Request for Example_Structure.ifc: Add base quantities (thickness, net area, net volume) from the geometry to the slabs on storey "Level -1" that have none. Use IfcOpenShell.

First a look at what the model holds.

```python
import ifcopenshell
import ifcopenshell.util.element
import ifcopenshell.util.unit

model = ifcopenshell.open("Example_Structure.ifc")
print(model.schema)
for unit_type in ("LENGTHUNIT", "AREAUNIT", "VOLUMEUNIT"):
    print(unit_type, ifcopenshell.util.unit.calculate_unit_scale(model, unit_type))
storey = next(s for s in model.by_type("IfcBuildingStorey") if s.Name == "Level -1")
slabs = [e for e in ifcopenshell.util.element.get_decomposition(storey) if e.is_a("IfcSlab")]
for e in sorted(slabs, key=lambda e: e.id()):
    print(e.id(), e.is_a(), e.Name, list(ifcopenshell.util.element.get_psets(e, qtos_only=True)), sep=" | ")
```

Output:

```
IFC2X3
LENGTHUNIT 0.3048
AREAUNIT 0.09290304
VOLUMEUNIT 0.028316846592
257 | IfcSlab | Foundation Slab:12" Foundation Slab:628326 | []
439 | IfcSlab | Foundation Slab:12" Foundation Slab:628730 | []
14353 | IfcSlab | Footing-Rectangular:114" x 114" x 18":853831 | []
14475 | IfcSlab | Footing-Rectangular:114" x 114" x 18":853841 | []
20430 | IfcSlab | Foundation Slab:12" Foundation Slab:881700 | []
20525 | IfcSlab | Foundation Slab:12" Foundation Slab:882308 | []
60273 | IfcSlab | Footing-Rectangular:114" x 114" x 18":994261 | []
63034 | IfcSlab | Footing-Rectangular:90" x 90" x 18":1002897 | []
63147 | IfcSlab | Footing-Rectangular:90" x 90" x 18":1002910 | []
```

```python
import ifcopenshell
import ifcopenshell.api.pset
import ifcopenshell.geom
import ifcopenshell.util.element
import ifcopenshell.util.shape
import ifcopenshell.util.unit

model = ifcopenshell.open("Example_Structure.ifc")
unit_scale = ifcopenshell.util.unit.calculate_unit_scale(model)
area_scale = ifcopenshell.util.unit.calculate_unit_scale(model, "AREAUNIT")
volume_scale = ifcopenshell.util.unit.calculate_unit_scale(model, "VOLUMEUNIT")
settings = ifcopenshell.geom.settings()

storey = next(s for s in model.by_type("IfcBuildingStorey") if s.Name == "Level -1")
slabs = [e for e in ifcopenshell.util.element.get_decomposition(storey) if e.is_a("IfcSlab")]

for e in sorted(slabs, key=lambda e: e.id()):
    if ifcopenshell.util.element.get_psets(e, qtos_only=True, should_inherit=False):
        continue
    # Geometry comes back in metres, in the element's own axes.
    shape = ifcopenshell.geom.create_shape(settings, e)
    values = {
        "Width": ifcopenshell.util.shape.get_z(shape.geometry) / unit_scale,
        "NetArea": ifcopenshell.util.shape.get_footprint_area(shape.geometry) / area_scale,
        "NetVolume": ifcopenshell.util.shape.get_volume(shape.geometry) / volume_scale,
    }
    qto = ifcopenshell.api.pset.add_qto(model, product=e, name="BaseQuantities")
    ifcopenshell.api.pset.edit_qto(model, qto=qto, properties=values)
    print(e.id(), {k: round(v, 3) for k, v in values.items()})

model.write("Example_Structure_rev.ifc")
```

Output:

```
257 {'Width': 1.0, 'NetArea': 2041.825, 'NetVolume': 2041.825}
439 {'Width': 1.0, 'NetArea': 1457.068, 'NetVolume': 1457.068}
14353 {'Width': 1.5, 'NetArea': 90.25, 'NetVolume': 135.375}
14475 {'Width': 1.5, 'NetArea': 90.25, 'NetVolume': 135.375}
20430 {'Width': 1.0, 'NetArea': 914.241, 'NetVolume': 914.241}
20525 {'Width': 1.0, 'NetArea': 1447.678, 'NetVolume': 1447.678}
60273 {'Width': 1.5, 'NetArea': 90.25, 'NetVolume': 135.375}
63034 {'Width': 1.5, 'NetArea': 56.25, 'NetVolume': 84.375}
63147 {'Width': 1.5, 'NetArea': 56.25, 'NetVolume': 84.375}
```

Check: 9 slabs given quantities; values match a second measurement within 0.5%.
